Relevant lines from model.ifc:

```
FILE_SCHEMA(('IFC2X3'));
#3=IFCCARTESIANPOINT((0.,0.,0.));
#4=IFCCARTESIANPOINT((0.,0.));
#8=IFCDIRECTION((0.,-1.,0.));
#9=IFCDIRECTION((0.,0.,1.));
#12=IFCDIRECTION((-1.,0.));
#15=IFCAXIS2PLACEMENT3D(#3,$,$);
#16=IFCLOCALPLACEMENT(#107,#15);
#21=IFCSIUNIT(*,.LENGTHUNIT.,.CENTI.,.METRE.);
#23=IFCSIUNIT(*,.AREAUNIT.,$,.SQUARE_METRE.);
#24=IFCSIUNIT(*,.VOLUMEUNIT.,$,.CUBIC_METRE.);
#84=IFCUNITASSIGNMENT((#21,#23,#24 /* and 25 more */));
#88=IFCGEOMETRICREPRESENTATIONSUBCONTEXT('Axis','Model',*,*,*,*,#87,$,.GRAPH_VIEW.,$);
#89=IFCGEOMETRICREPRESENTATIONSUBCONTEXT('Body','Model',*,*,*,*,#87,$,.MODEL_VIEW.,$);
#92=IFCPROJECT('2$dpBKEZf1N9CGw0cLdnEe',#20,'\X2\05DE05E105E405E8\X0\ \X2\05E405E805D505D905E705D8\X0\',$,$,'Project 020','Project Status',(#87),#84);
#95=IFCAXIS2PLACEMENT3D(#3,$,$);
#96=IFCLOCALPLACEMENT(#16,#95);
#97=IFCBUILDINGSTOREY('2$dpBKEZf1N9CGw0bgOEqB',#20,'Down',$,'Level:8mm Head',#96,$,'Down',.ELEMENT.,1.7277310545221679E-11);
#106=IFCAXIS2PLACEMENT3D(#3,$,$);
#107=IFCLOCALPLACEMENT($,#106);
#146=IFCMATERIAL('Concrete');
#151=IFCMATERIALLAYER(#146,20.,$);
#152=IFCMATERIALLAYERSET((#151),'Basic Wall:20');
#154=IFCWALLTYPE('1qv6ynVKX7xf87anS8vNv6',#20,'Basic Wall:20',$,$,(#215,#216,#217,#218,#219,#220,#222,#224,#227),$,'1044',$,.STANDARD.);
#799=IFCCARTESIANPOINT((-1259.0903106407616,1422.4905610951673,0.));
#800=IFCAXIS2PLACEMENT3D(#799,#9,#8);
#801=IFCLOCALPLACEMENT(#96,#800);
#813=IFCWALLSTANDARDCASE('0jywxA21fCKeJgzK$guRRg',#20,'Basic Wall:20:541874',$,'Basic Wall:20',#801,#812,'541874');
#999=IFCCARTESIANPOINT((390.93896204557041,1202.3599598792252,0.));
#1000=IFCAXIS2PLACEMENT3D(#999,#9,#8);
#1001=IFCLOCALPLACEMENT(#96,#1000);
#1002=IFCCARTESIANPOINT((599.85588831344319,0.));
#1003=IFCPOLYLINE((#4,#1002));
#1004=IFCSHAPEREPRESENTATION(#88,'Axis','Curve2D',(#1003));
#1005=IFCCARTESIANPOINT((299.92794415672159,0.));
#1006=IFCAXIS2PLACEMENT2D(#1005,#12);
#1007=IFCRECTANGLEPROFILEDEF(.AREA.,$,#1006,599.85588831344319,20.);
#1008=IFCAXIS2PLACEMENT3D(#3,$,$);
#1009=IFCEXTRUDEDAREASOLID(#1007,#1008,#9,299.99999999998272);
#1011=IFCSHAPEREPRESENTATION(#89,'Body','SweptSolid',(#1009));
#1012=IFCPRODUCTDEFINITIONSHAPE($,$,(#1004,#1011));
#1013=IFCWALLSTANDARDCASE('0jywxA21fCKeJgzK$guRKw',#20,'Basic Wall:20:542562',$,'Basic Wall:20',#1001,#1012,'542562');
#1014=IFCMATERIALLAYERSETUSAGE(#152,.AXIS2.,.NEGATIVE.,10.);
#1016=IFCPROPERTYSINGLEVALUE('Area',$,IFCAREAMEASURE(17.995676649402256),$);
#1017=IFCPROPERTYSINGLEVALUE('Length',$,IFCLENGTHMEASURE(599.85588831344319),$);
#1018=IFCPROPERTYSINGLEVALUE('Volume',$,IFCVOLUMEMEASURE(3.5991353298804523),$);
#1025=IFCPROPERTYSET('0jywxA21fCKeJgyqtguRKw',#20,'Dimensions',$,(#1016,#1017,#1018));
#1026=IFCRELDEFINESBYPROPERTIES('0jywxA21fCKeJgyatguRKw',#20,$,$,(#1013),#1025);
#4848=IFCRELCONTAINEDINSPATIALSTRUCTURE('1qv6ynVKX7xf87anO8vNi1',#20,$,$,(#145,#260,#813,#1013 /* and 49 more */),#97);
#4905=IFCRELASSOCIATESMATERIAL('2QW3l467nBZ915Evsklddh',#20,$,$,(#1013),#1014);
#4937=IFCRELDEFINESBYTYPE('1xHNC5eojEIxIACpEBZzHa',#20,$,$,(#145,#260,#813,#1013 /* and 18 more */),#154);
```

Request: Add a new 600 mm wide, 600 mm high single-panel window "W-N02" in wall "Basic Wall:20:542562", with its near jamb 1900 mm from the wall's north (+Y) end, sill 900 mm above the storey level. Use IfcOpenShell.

```python
import numpy as np
import ifcopenshell
import ifcopenshell.api.feature
import ifcopenshell.api.geometry
import ifcopenshell.api.pset
import ifcopenshell.api.root
import ifcopenshell.api.spatial
import ifcopenshell.api.type
import ifcopenshell.geom
import ifcopenshell.util.element
import ifcopenshell.util.placement
import ifcopenshell.util.representation
import ifcopenshell.util.shape
import ifcopenshell.util.unit

model = ifcopenshell.open("model.ifc")
unit_scale = ifcopenshell.util.unit.calculate_unit_scale(model)
area_scale = ifcopenshell.util.unit.calculate_unit_scale(model, "AREAUNIT")
volume_scale = ifcopenshell.util.unit.calculate_unit_scale(model, "VOLUMEUNIT")
settings = ifcopenshell.geom.settings()


def volume(element):
    """Net volume in cubic metres, openings subtracted."""
    shape = ifcopenshell.geom.create_shape(settings, element)
    return ifcopenshell.util.shape.get_volume(shape.geometry)


wall = model.by_guid("0jywxA21fCKeJgzK$guRKw")
storey = ifcopenshell.util.element.get_container(wall, ifc_class="IfcBuildingStorey")
context = ifcopenshell.util.representation.get_context(model, "Model", "Body", "MODEL_VIEW")
before = volume(wall)

width, height, from_end, sill = 0.6, 0.6, 1.9, 0.9  # metres

# The wall runs along its own X axis, and the end named is its -X end.
wall_shape = ifcopenshell.geom.create_shape(settings, wall)
x, y, z = ifcopenshell.util.shape.get_vertices(wall_shape.geometry).T
start = x.min() + from_end
face, thickness = float(y.min()), float(y.max() - y.min())
wall_matrix = ifcopenshell.util.placement.get_local_placement(wall.ObjectPlacement)
level = ifcopenshell.util.placement.get_local_placement(storey.ObjectPlacement)[2, 3]


def in_wall(x, y):
    """Placement at x, y metres in the wall's axes, at sill height."""
    matrix = wall_matrix.copy()
    matrix[:, 3] = wall_matrix @ np.array([x / unit_scale, y / unit_scale, 0.0, 1.0])
    matrix[2, 3] = level + sill / unit_scale
    return matrix


# Opening: a box that overshoots both wall faces by 50 mm.
opening = ifcopenshell.api.root.create_entity(model, ifc_class="IfcOpeningElement")
box = ifcopenshell.api.geometry.add_wall_representation(
    model, context=context, length=width, height=height, thickness=thickness + 0.1
)
ifcopenshell.api.geometry.assign_representation(model, product=opening, representation=box)
ifcopenshell.api.geometry.edit_object_placement(model, product=opening, matrix=in_wall(start, face - 0.05), is_si=False)
ifcopenshell.api.feature.add_feature(model, feature=opening, element=wall)

window = ifcopenshell.api.root.create_entity(model, ifc_class="IfcWindow", name="W-N02")
window.OverallWidth, window.OverallHeight = width / unit_scale, height / unit_scale
body = ifcopenshell.api.geometry.add_window_representation(
    model,
    context=context,
    overall_width=window.OverallWidth,
    overall_height=window.OverallHeight,
    partition_type="SINGLE_PANEL",
)
ifcopenshell.api.geometry.assign_representation(model, product=window, representation=body)
ifcopenshell.api.spatial.assign_container(model, products=[window], relating_structure=storey)
fills = ifcopenshell.api.feature.add_filling(model, opening=opening, element=window)
fills.OwnerHistory = window.OwnerHistory  # required in IFC2X3

# IFC2X3 keeps the operation on the window style.
style = ifcopenshell.api.root.create_entity(model, ifc_class="IfcWindowStyle", name="W-N02")
style.OperationType, style.ConstructionType = "SINGLE_PANEL", "NOTDEFINED"
style.ParameterTakesPrecedence = style.Sizeable = False
ifcopenshell.api.type.assign_type(model, related_objects=[window], relating_type=style)

# Centre the window in the wall's thickness.
ifcopenshell.api.geometry.edit_object_placement(model, product=window, matrix=in_wall(start, face), is_si=False)
window_shape = ifcopenshell.geom.create_shape(settings, window)
depth = ifcopenshell.util.shape.get_vertices(window_shape.geometry)[:, 1]
offset = face + thickness / 2 - (depth.min() + depth.max()) / 2
ifcopenshell.api.geometry.edit_object_placement(model, product=window, matrix=in_wall(start, offset), is_si=False)

after = volume(wall)

# Update the wall's stored quantities.
pset = model.by_id(ifcopenshell.util.element.get_pset(wall, "Dimensions", should_inherit=False)["id"])
ifcopenshell.api.pset.edit_pset(model, pset=pset, properties={
    "Area": model.create_entity("IfcAreaMeasure", after / thickness / area_scale),
    "Volume": model.create_entity("IfcVolumeMeasure", after / volume_scale),
})

print(f"wall volume {before:.3f} -> {after:.3f} m3")

model.write("model_updated.ifc")
```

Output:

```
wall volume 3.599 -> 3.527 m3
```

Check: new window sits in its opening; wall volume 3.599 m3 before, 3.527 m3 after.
